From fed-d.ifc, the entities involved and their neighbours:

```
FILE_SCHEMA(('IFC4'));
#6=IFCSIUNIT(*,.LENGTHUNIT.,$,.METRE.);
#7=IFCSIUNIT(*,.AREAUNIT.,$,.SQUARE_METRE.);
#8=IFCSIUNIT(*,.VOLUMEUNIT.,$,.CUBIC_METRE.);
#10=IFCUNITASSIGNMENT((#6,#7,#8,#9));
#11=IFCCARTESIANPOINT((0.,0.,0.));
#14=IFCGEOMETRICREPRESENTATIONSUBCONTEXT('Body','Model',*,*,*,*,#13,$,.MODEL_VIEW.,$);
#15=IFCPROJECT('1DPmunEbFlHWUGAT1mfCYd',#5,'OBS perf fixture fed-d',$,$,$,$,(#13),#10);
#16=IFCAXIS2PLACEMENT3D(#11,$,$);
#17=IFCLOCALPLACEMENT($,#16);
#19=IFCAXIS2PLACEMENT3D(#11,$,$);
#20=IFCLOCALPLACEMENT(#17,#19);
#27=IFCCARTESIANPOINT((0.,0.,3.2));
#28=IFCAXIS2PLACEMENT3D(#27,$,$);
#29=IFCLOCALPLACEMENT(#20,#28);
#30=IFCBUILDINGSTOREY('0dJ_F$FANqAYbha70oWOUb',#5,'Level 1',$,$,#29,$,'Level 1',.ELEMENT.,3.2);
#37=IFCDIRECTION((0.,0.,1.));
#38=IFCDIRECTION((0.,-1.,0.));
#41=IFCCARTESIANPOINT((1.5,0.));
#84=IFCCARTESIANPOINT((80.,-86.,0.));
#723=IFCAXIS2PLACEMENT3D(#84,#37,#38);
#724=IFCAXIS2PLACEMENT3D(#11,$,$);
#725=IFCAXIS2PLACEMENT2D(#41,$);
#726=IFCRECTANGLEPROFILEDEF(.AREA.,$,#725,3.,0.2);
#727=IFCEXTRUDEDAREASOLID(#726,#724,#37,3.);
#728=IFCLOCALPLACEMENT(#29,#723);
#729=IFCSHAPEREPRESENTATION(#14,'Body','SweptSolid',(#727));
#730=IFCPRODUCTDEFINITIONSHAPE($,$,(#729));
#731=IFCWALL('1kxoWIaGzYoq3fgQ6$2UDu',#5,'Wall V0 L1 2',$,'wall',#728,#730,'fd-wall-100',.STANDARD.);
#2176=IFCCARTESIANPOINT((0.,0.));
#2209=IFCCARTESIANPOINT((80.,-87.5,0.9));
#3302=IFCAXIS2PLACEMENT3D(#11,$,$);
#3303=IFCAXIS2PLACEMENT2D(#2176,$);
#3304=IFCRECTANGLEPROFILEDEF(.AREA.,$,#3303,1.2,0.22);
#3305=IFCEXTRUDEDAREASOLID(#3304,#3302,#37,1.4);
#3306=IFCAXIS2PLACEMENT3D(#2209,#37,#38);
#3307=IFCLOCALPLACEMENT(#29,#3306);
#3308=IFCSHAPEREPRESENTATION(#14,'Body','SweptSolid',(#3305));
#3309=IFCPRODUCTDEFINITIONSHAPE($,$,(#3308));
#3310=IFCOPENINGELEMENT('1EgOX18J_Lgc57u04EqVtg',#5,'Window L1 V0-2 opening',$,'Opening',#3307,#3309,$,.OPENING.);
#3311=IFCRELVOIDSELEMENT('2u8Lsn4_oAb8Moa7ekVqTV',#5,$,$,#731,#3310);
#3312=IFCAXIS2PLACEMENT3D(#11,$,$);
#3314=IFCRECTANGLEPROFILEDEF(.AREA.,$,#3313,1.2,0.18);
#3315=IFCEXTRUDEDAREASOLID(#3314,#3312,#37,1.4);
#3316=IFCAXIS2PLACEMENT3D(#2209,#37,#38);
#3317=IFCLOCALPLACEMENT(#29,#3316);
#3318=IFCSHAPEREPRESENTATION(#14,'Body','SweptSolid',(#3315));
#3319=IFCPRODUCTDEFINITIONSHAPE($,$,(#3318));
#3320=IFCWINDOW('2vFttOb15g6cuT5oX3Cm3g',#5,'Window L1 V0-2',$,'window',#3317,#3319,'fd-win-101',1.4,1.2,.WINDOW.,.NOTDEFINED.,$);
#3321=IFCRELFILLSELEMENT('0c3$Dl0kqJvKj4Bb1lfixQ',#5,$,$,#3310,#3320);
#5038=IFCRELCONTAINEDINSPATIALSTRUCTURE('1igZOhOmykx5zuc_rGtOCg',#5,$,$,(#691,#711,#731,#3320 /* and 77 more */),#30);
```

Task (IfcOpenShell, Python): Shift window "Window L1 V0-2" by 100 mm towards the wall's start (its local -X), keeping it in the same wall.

```python
import ifcopenshell
import ifcopenshell.api.geometry
import ifcopenshell.util.placement
import ifcopenshell.util.unit

model = ifcopenshell.open("fed-d.ifc")
unit_scale = ifcopenshell.util.unit.calculate_unit_scale(model)

window = model.by_guid("2vFttOb15g6cuT5oX3Cm3g")
opening = window.FillsVoids[0].RelatingOpeningElement
wall = opening.VoidsElements[0].RelatingBuildingElement

wall_matrix = ifcopenshell.util.placement.get_local_placement(wall.ObjectPlacement)
shift = wall_matrix[:3, 0] * -0.1 / unit_scale
before = ifcopenshell.util.placement.get_local_placement(window.ObjectPlacement)[:3, 3].copy()

# The window is not placed relative to its opening, so move both.
for product in (opening, window):
    matrix = ifcopenshell.util.placement.get_local_placement(product.ObjectPlacement)
    matrix[:3, 3] += shift
    ifcopenshell.api.geometry.edit_object_placement(model, product=product, matrix=matrix, is_si=False)

after = ifcopenshell.util.placement.get_local_placement(window.ObjectPlacement)[:3, 3]
print("window moved by", (after - before).round(3) + 0.0)

model.write("fed-d_edited.ifc")
```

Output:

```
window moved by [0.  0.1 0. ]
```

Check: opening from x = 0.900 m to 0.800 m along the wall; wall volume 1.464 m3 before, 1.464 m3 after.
